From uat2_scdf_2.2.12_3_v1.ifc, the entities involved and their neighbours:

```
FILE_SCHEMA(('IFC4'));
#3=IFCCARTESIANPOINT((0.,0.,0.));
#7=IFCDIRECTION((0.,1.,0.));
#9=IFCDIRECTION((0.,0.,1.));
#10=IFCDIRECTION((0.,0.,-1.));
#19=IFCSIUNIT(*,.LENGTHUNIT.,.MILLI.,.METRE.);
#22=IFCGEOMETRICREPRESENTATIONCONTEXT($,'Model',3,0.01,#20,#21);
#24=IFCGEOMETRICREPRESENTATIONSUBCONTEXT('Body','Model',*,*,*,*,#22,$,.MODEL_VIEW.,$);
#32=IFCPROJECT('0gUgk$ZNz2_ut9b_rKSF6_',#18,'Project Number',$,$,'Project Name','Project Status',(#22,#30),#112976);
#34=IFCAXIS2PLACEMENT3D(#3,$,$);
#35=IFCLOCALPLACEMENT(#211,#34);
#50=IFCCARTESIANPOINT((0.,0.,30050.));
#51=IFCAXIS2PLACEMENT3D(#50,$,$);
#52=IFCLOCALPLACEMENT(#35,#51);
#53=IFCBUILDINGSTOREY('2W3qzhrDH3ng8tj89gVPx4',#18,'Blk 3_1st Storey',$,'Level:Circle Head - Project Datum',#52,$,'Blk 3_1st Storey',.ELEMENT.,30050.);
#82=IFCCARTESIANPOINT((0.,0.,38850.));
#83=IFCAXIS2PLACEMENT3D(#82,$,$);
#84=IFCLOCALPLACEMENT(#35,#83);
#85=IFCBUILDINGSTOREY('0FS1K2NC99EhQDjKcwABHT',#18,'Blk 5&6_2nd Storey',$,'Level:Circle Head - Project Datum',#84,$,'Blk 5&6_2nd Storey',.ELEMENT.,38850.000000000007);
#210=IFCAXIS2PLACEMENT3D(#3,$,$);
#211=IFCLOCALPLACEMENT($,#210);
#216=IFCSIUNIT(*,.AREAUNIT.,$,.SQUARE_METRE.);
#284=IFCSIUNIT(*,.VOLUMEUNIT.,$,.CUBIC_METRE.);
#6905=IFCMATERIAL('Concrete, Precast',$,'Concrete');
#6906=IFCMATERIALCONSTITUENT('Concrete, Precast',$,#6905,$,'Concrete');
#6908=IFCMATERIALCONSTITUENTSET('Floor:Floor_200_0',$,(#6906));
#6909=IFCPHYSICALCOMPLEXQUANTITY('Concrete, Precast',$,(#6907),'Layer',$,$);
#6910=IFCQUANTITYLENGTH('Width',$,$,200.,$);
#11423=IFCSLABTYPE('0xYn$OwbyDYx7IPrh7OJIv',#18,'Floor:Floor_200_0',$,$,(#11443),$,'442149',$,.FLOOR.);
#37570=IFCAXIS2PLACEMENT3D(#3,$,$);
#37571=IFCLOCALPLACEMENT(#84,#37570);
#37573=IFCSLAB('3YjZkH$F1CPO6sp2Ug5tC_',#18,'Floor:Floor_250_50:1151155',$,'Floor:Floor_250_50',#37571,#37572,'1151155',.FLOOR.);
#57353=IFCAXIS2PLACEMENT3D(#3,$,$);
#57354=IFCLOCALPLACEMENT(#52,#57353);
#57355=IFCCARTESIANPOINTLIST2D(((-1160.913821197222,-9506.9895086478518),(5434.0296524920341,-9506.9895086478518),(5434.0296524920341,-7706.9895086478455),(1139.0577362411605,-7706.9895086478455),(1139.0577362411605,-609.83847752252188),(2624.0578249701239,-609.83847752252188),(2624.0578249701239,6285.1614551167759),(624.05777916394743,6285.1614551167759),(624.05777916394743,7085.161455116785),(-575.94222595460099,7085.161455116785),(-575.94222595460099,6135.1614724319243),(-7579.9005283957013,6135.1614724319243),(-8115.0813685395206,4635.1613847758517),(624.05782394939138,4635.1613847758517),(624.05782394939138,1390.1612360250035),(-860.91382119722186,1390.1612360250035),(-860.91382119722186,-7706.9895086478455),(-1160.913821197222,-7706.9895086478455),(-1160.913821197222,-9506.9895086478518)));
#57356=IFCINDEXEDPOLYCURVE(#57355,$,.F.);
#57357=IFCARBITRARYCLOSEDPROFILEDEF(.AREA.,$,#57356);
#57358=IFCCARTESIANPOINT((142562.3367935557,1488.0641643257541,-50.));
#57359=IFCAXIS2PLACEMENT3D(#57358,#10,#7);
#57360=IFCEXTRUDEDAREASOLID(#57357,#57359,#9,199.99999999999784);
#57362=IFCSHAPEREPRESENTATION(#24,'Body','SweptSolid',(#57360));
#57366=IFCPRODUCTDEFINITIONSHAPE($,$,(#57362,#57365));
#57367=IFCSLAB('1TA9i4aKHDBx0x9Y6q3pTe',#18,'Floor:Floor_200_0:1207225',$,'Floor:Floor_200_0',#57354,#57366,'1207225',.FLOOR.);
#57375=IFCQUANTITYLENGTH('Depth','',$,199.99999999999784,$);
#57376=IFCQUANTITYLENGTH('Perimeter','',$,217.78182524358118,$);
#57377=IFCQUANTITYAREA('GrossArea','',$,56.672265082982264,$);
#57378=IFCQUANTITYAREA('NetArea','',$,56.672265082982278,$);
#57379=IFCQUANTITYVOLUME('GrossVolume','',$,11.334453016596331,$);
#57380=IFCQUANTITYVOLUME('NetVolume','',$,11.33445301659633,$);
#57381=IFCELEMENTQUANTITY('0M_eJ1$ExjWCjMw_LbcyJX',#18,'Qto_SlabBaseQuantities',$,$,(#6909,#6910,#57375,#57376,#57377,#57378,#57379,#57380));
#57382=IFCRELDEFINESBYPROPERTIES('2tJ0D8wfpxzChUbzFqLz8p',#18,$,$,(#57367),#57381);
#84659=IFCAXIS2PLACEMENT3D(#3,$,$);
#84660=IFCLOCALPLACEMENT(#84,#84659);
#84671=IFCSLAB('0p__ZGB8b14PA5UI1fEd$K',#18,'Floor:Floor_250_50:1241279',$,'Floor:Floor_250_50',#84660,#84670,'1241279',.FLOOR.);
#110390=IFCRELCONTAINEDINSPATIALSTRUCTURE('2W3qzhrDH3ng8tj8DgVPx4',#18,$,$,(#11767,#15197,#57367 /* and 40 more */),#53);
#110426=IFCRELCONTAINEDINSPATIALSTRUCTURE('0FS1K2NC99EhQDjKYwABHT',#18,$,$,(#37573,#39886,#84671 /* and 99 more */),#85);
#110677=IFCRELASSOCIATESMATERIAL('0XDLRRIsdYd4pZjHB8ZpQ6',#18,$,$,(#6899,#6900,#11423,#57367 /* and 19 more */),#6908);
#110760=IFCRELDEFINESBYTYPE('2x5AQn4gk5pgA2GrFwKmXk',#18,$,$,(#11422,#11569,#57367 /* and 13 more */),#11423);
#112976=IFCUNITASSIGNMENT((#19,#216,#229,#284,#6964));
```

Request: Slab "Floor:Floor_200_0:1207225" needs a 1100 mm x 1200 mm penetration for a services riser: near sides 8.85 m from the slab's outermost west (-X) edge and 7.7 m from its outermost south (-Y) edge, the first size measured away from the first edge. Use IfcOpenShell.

```python
import numpy as np
import ifcopenshell
import ifcopenshell.api.feature
import ifcopenshell.api.geometry
import ifcopenshell.api.pset
import ifcopenshell.api.root
import ifcopenshell.geom
import ifcopenshell.util.element
import ifcopenshell.util.placement
import ifcopenshell.util.representation
import ifcopenshell.util.shape
import ifcopenshell.util.unit

model = ifcopenshell.open("uat2_scdf_2.2.12_3_v1.ifc")
unit_scale = ifcopenshell.util.unit.calculate_unit_scale(model)
area_scale = ifcopenshell.util.unit.calculate_unit_scale(model, "AREAUNIT")
volume_scale = ifcopenshell.util.unit.calculate_unit_scale(model, "VOLUMEUNIT")
settings = ifcopenshell.geom.settings()


def volume(element):
    """Net volume in cubic metres, openings subtracted."""
    shape = ifcopenshell.geom.create_shape(settings, element)
    return ifcopenshell.util.shape.get_volume(shape.geometry)


slab = model.by_id(57367)
before = volume(slab)

# Extent in the slab's own axes, in metres. The edges named are its -X and -Y sides.
slab_shape = ifcopenshell.geom.create_shape(settings, slab)
vertices = ifcopenshell.util.shape.get_vertices(slab_shape.geometry)
x_min, y_min, bottom = vertices.min(axis=0)
top = vertices[:, 2].max()

opening = ifcopenshell.api.root.create_entity(model, ifc_class="IfcOpeningElement", name="Services riser opening", predefined_type="OPENING")
context = ifcopenshell.util.representation.get_context(model, "Model", "Body", "MODEL_VIEW")
width, depth = 1.1, 1.2
outline = [(0.0, 0.0), (width, 0.0), (width, depth), (0.0, depth), (0.0, 0.0)]
# Overshoot both faces by 50 mm so the cut is clean.
shape = ifcopenshell.api.geometry.add_slab_representation(
    model, context=context, depth=top - bottom + 0.1, polyline=outline
)
ifcopenshell.api.geometry.assign_representation(model, product=opening, representation=shape)

matrix = ifcopenshell.util.placement.get_local_placement(slab.ObjectPlacement)
matrix[:, 3] = matrix @ np.append(np.array([x_min + 8.85, y_min + 7.7, bottom - 0.05]) / unit_scale, 1.0)
ifcopenshell.api.geometry.edit_object_placement(model, product=opening, matrix=matrix, is_si=False)
ifcopenshell.api.feature.add_feature(model, feature=opening, element=slab)

after = volume(slab)

# Update the slab's stored quantities.
qto = model.by_id(ifcopenshell.util.element.get_pset(slab, "Qto_SlabBaseQuantities", should_inherit=False)["id"])
ifcopenshell.api.pset.edit_qto(model, qto=qto, properties={
    "NetArea": after / (top - bottom) / area_scale,
    "NetVolume": after / volume_scale,
})

print(f"slab volume {before:.3f} -> {after:.3f} m3")

model.write("uat2_scdf_2.2.12_3_v1_v2.ifc")
```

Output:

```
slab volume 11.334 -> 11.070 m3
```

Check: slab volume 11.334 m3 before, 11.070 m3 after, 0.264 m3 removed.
